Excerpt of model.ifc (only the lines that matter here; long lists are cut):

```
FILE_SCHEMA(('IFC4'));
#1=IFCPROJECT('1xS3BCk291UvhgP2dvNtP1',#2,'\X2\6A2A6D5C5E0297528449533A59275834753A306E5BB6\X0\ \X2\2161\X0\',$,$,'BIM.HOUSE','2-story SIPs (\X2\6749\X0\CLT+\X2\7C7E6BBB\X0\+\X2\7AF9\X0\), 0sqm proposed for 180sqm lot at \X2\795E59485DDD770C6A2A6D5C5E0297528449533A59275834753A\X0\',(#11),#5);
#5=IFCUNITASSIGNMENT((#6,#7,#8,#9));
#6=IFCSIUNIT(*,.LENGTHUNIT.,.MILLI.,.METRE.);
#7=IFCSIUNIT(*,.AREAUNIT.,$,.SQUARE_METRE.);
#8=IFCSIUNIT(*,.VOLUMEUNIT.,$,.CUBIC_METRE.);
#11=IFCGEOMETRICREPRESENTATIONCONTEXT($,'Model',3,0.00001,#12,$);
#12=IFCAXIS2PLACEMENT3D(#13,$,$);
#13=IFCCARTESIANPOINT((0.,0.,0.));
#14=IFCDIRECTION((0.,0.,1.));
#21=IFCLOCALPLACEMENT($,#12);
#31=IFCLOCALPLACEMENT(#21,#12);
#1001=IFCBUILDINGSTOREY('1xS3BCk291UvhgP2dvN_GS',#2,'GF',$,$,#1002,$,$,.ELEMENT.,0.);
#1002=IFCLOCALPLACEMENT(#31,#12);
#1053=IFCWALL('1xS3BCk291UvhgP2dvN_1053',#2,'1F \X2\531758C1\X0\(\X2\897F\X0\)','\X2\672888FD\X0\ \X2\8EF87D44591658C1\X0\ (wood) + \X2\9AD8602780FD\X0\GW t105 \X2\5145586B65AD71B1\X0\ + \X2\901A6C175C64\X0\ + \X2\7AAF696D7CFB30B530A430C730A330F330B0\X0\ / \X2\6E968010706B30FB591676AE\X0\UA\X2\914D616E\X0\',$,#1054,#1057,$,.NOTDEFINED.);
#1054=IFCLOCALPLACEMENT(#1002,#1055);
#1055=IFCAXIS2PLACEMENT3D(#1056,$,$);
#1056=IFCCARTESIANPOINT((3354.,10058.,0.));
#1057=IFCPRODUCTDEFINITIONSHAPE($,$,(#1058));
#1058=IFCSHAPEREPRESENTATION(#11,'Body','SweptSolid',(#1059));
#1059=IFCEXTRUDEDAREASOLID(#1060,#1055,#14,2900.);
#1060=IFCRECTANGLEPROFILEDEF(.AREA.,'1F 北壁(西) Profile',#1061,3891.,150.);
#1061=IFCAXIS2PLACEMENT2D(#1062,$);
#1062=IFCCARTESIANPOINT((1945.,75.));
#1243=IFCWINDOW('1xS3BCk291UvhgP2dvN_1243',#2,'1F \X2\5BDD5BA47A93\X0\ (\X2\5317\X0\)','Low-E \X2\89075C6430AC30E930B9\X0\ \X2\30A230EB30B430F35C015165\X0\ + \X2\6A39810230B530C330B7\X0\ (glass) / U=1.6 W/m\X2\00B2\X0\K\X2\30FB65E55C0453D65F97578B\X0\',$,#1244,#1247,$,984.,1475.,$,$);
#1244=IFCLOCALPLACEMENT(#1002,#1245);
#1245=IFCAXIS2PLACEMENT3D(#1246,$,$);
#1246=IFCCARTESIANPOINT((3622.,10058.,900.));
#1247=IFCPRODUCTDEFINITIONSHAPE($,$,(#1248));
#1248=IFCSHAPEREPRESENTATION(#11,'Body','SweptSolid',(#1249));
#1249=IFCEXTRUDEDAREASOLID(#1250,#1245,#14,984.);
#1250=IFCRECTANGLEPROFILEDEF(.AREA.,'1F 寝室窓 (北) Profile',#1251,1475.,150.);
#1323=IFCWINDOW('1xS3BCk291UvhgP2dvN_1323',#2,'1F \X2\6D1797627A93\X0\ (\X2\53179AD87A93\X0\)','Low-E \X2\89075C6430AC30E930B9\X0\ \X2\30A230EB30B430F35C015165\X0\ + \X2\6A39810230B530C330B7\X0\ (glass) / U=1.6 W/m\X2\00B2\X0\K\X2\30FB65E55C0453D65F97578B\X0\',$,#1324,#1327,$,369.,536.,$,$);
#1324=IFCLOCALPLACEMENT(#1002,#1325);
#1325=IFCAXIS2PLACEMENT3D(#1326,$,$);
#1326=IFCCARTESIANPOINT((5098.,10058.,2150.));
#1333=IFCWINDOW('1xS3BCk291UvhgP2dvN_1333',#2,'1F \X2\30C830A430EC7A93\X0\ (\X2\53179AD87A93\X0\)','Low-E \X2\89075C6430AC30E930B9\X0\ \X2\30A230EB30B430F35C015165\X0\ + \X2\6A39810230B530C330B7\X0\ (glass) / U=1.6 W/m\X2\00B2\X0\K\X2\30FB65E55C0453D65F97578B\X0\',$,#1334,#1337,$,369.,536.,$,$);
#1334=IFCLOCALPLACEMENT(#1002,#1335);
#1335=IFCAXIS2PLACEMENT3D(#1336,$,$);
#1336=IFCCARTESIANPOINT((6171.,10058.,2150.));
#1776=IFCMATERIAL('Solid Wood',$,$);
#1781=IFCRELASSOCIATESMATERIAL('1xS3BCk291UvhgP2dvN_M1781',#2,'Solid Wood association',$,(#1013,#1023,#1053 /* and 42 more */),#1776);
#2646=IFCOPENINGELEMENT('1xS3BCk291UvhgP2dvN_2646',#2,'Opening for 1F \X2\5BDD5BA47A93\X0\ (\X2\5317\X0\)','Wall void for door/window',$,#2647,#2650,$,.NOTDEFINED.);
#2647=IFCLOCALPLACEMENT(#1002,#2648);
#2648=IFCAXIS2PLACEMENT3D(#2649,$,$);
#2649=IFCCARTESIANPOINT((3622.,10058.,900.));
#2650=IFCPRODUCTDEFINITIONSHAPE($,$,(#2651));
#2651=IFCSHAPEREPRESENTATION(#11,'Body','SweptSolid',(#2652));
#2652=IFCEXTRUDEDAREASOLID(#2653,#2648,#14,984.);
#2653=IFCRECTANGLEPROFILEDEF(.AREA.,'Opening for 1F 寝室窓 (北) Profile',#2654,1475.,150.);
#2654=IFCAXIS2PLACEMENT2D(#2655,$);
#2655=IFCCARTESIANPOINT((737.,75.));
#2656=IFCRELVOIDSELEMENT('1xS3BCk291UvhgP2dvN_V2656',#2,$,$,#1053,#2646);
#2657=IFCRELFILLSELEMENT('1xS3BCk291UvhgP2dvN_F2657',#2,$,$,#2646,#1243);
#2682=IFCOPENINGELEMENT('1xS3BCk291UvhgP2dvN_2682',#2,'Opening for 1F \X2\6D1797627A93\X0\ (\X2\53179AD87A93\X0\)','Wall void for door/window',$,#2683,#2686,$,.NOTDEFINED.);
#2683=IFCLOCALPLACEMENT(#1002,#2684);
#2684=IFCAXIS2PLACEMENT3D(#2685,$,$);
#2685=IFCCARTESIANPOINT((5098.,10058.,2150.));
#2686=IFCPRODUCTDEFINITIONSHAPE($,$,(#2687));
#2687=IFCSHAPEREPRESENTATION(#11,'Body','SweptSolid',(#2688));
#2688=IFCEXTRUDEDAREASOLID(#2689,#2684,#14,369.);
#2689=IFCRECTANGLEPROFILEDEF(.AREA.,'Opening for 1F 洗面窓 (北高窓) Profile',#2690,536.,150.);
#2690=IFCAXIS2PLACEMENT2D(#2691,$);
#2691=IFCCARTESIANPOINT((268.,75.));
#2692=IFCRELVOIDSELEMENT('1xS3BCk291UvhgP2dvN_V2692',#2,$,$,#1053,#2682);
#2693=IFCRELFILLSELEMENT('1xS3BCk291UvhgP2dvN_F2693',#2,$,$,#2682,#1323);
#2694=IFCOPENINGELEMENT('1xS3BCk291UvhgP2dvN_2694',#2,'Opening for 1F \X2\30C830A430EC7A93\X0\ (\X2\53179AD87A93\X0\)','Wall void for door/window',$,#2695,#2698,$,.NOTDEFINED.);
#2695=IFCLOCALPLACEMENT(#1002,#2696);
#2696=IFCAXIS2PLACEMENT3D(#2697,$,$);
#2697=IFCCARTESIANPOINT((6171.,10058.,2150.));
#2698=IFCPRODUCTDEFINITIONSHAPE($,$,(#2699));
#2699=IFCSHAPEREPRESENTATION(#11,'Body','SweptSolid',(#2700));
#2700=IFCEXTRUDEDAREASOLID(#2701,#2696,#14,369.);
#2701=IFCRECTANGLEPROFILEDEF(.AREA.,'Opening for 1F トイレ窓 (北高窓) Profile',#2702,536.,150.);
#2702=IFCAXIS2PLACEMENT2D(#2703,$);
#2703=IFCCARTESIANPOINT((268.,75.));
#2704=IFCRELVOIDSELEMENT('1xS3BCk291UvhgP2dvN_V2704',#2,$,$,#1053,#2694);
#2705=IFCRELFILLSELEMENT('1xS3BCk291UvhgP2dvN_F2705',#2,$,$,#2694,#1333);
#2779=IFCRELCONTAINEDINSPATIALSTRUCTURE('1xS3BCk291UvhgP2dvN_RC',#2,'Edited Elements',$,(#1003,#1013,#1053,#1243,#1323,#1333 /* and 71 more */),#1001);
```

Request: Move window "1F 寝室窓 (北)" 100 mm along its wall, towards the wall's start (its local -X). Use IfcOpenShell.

```python
import ifcopenshell
import ifcopenshell.api.geometry
import ifcopenshell.util.placement
import ifcopenshell.util.unit

model = ifcopenshell.open("model.ifc")
unit_scale = ifcopenshell.util.unit.calculate_unit_scale(model)

window = model.by_id(1243)
opening = window.FillsVoids[0].RelatingOpeningElement
wall = opening.VoidsElements[0].RelatingBuildingElement

wall_matrix = ifcopenshell.util.placement.get_local_placement(wall.ObjectPlacement)
shift = wall_matrix[:3, 0] * -0.1 / unit_scale
before = ifcopenshell.util.placement.get_local_placement(window.ObjectPlacement)[:3, 3].copy()

# The window is not placed relative to its opening, so move both.
for product in (opening, window):
    matrix = ifcopenshell.util.placement.get_local_placement(product.ObjectPlacement)
    matrix[:3, 3] += shift
    ifcopenshell.api.geometry.edit_object_placement(model, product=product, matrix=matrix, is_si=False)

after = ifcopenshell.util.placement.get_local_placement(window.ObjectPlacement)[:3, 3]
print("window moved by", (after - before).round(3) + 0.0)

model.write("model_rev.ifc")
```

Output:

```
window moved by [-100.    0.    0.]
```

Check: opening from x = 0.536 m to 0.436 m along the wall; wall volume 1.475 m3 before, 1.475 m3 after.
